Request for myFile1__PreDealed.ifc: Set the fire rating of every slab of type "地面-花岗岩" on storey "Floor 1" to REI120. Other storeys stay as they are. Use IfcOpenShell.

First a look at what the model holds.

```python
import ifcopenshell
import ifcopenshell.util.element

model = ifcopenshell.open("myFile1__PreDealed.ifc")
print(model.schema)
storey = next(s for s in model.by_type("IfcBuildingStorey") if s.Name == "Floor 1")
slabs = [e for e in ifcopenshell.util.element.get_decomposition(storey) if e.is_a("IfcSlab")]
seen = {}
for e in slabs:
    element_type = ifcopenshell.util.element.get_type(e)
    key = (element_type.Name if element_type != e and element_type else None, ifcopenshell.util.element.get_pset(e, "Pset_SlabCommon", "FireRating"))
    seen[key] = seen.get(key, 0) + 1
for (name, value), count in sorted(seen.items(), key=str):
    print(count, "x", name, "|", value)
```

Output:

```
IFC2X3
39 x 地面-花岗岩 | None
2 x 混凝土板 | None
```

```python
import ifcopenshell
import ifcopenshell.api.pset
import ifcopenshell.util.element

model = ifcopenshell.open("myFile1__PreDealed.ifc")

storey = next(s for s in model.by_type("IfcBuildingStorey") if s.Name == "Floor 1")
slabs = [e for e in ifcopenshell.util.element.get_decomposition(storey) if e.is_a("IfcSlab")]

count = 0
for e in slabs:
    element_type = ifcopenshell.util.element.get_type(e)
    if element_type in (None, e) or element_type.Name != "地面-花岗岩":
        continue
    # add_pset returns the element's existing set when there is one.
    pset = ifcopenshell.api.pset.add_pset(model, product=e, name="Pset_SlabCommon")
    ifcopenshell.api.pset.edit_pset(model, pset=pset, properties={"FireRating": "REI120"})
    count += 1

print(count, "slabs updated")

model.write("myFile1__PreDealed_rev.ifc")
```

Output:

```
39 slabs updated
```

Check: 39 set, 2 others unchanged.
